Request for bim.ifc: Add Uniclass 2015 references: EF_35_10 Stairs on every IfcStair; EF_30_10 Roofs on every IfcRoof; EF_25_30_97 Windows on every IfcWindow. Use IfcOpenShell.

First a look at what the model holds.

```python
import ifcopenshell

model = ifcopenshell.open("bim.ifc")
print(model.schema)
print("classifications:", [c.Name for c in model.by_type("IfcClassification")])
for ifc_class in ("IfcDoor", "IfcRoof", "IfcStair", "IfcWall", "IfcWindow"):
    print(ifc_class, len(model.by_type(ifc_class)))
```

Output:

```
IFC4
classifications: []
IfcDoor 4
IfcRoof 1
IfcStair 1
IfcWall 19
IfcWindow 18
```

```python
import ifcopenshell
import ifcopenshell.api.classification

model = ifcopenshell.open("bim.ifc")

system = ifcopenshell.api.classification.add_classification(model, classification="Uniclass 2015")

codes = {
    "IfcStair": ("EF_35_10", "Stairs"),
    "IfcRoof": ("EF_30_10", "Roofs"),
    "IfcWindow": ("EF_25_30_97", "Windows"),
}
for ifc_class, (code, name) in codes.items():
    products = model.by_type(ifc_class)
    ifcopenshell.api.classification.add_reference(
        model, products=products, classification=system, identification=code, name=name
    )
    print(code, len(products))

model.write("bim_updated.ifc")
```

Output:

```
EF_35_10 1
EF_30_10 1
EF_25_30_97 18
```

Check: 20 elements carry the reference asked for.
